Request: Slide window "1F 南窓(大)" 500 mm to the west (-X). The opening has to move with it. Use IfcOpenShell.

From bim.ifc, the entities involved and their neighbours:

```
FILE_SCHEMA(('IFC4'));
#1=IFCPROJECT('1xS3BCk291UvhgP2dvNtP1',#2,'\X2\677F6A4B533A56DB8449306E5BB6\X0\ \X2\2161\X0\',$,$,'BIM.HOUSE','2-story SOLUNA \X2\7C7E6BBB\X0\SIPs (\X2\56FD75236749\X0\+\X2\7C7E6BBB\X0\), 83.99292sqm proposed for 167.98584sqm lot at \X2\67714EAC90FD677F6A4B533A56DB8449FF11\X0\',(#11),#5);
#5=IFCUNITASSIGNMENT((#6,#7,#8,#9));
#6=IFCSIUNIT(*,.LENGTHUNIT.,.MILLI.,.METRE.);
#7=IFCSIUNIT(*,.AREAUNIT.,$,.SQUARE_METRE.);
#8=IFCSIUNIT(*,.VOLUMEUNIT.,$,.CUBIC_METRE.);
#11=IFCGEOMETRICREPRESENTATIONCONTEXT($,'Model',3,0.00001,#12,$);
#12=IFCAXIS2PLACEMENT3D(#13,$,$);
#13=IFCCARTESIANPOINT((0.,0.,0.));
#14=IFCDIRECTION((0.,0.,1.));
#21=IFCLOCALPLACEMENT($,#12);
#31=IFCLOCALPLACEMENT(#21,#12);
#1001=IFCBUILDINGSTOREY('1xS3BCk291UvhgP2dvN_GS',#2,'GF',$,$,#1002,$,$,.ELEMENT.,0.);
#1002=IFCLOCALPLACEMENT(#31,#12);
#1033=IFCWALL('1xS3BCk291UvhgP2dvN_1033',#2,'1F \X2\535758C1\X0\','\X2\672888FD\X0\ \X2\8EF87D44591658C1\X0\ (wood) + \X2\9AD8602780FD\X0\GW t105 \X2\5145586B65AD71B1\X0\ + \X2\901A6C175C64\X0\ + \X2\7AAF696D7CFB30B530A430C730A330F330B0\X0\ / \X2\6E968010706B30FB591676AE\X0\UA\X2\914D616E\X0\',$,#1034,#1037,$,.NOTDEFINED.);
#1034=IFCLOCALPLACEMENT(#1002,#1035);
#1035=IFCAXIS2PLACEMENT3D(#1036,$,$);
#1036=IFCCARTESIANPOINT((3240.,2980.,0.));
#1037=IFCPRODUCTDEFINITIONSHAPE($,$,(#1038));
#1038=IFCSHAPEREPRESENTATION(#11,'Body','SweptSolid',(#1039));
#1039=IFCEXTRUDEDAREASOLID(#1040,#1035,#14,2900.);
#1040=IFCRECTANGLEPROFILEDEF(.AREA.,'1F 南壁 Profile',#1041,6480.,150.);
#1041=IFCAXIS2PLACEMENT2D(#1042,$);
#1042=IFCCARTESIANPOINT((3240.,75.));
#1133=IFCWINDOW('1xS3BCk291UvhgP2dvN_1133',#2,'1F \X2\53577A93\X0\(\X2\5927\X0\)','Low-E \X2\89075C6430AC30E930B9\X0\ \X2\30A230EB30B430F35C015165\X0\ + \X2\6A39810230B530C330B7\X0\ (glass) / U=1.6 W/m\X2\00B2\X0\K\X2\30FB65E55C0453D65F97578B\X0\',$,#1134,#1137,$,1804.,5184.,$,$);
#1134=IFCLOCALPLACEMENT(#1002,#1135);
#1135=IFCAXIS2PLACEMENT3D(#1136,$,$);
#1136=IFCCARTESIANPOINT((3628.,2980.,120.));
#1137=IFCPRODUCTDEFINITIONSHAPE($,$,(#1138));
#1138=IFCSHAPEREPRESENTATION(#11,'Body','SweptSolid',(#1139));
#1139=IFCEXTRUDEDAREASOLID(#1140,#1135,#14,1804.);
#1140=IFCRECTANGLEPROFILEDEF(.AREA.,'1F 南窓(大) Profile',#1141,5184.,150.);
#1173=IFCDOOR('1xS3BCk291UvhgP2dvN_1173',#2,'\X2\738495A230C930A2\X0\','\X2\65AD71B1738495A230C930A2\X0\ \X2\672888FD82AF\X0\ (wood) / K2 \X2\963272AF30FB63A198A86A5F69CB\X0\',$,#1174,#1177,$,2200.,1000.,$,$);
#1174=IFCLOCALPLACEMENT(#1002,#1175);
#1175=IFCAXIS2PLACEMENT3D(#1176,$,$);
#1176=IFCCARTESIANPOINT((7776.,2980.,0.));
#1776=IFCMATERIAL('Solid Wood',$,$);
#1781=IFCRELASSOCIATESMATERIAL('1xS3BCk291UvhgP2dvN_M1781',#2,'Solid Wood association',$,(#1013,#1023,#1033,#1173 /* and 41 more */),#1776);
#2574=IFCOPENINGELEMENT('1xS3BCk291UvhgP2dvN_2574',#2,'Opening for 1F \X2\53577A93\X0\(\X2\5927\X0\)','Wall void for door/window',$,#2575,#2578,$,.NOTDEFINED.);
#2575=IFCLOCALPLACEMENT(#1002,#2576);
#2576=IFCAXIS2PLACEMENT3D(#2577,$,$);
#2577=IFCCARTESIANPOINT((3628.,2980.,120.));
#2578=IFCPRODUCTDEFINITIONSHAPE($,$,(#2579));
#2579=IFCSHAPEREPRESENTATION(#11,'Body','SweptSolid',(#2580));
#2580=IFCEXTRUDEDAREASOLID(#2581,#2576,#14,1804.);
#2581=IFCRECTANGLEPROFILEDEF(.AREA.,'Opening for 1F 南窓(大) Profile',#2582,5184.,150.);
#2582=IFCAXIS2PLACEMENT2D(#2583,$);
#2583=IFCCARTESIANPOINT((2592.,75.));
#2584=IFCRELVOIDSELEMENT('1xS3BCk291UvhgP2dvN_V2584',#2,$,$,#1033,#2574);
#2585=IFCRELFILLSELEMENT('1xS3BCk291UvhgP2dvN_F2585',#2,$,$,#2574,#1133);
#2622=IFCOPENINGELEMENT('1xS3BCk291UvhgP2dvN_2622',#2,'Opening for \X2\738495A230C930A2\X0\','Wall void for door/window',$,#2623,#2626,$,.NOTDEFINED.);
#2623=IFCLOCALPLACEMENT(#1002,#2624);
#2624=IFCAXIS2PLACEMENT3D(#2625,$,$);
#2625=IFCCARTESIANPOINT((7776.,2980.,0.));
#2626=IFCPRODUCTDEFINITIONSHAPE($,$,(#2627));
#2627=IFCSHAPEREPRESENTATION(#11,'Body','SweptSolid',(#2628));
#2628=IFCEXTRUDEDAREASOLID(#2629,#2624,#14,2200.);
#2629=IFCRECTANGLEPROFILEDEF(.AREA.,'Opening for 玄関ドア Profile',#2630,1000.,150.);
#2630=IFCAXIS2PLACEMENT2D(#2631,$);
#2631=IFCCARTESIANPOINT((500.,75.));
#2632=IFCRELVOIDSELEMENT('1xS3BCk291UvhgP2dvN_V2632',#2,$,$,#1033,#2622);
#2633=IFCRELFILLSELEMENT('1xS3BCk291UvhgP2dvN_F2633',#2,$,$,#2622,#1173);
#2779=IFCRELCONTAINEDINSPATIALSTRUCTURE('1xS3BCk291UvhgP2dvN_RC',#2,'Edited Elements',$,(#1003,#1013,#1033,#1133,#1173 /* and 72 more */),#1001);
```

```python
import ifcopenshell
import ifcopenshell.api.geometry
import ifcopenshell.util.placement
import ifcopenshell.util.unit

model = ifcopenshell.open("bim.ifc")
unit_scale = ifcopenshell.util.unit.calculate_unit_scale(model)

window = model.by_guid("1xS3BCk291UvhgP2dvN_1133")
opening = window.FillsVoids[0].RelatingOpeningElement
wall = opening.VoidsElements[0].RelatingBuildingElement

wall_matrix = ifcopenshell.util.placement.get_local_placement(wall.ObjectPlacement)
shift = wall_matrix[:3, 0] * -0.5 / unit_scale
before = ifcopenshell.util.placement.get_local_placement(window.ObjectPlacement)[:3, 3].copy()

# The window is not placed relative to its opening, so move both.
for product in (opening, window):
    matrix = ifcopenshell.util.placement.get_local_placement(product.ObjectPlacement)
    matrix[:3, 3] += shift
    ifcopenshell.api.geometry.edit_object_placement(model, product=product, matrix=matrix, is_si=False)

after = ifcopenshell.util.placement.get_local_placement(window.ObjectPlacement)[:3, 3]
print("window moved by", (after - before).round(3) + 0.0)

model.write("bim_edited.ifc")
```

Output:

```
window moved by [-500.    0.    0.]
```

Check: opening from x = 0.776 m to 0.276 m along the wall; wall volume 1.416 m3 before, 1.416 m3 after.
